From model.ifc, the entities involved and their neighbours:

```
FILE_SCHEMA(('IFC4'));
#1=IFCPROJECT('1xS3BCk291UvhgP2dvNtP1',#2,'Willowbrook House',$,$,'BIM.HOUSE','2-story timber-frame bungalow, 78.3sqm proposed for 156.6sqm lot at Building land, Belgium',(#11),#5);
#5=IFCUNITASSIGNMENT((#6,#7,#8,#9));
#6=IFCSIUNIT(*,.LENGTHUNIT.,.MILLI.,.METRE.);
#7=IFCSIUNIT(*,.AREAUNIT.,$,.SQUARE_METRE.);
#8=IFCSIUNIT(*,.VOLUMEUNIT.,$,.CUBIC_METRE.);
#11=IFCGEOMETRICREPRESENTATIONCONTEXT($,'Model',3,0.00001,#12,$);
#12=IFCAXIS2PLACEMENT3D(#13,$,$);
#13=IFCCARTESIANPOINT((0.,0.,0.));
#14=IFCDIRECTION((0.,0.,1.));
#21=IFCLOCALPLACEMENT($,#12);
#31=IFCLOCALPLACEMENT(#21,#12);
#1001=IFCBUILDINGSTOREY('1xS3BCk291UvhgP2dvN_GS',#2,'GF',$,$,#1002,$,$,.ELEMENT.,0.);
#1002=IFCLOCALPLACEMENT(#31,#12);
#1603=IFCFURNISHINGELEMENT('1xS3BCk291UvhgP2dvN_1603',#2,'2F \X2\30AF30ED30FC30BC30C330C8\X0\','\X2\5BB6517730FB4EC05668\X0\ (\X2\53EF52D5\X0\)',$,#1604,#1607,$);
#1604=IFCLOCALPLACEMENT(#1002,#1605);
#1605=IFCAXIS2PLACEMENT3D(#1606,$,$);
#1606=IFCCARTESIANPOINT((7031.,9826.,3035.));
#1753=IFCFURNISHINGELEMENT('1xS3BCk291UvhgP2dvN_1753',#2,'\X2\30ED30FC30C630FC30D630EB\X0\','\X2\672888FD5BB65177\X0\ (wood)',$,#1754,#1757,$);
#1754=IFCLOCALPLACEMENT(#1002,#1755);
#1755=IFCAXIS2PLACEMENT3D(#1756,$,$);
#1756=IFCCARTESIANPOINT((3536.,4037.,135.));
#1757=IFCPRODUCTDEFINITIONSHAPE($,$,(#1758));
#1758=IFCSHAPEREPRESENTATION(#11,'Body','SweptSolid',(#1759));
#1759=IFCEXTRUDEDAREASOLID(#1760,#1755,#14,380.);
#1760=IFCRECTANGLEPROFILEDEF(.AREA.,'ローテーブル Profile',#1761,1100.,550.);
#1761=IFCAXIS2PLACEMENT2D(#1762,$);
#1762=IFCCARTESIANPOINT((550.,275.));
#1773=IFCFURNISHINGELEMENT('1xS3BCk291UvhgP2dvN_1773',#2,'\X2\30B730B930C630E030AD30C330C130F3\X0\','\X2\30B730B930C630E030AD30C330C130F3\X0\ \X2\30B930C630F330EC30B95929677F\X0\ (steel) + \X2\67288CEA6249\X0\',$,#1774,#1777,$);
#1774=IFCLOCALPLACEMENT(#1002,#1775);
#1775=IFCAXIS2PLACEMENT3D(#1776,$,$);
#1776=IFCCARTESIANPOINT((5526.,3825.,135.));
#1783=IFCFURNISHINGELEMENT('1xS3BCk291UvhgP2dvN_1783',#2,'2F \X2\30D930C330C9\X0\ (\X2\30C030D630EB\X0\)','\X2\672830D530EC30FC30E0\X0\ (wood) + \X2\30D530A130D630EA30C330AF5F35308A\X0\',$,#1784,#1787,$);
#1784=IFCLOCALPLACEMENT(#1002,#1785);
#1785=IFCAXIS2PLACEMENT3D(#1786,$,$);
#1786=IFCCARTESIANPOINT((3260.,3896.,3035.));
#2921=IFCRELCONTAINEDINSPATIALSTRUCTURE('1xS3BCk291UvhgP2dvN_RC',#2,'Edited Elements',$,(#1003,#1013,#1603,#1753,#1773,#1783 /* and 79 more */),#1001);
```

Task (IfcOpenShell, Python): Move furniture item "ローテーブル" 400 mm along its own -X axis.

```python
import ifcopenshell
import ifcopenshell.api.geometry
import ifcopenshell.util.placement
import ifcopenshell.util.unit

model = ifcopenshell.open("model.ifc")
unit_scale = ifcopenshell.util.unit.calculate_unit_scale(model)

item = model.by_id(1753)
matrix = ifcopenshell.util.placement.get_local_placement(item.ObjectPlacement)
matrix[:3, 3] -= matrix[:3, 0] * 0.4 / unit_scale
ifcopenshell.api.geometry.edit_object_placement(model, product=item, matrix=matrix, is_si=False)

print(ifcopenshell.util.placement.get_local_placement(item.ObjectPlacement).round(3) + 0.0)

model.write("model_edited.ifc")
```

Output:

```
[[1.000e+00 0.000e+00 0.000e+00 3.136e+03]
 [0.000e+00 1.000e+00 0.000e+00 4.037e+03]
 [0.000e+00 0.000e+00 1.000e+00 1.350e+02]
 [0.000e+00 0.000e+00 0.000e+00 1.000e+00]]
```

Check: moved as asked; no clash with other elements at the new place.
